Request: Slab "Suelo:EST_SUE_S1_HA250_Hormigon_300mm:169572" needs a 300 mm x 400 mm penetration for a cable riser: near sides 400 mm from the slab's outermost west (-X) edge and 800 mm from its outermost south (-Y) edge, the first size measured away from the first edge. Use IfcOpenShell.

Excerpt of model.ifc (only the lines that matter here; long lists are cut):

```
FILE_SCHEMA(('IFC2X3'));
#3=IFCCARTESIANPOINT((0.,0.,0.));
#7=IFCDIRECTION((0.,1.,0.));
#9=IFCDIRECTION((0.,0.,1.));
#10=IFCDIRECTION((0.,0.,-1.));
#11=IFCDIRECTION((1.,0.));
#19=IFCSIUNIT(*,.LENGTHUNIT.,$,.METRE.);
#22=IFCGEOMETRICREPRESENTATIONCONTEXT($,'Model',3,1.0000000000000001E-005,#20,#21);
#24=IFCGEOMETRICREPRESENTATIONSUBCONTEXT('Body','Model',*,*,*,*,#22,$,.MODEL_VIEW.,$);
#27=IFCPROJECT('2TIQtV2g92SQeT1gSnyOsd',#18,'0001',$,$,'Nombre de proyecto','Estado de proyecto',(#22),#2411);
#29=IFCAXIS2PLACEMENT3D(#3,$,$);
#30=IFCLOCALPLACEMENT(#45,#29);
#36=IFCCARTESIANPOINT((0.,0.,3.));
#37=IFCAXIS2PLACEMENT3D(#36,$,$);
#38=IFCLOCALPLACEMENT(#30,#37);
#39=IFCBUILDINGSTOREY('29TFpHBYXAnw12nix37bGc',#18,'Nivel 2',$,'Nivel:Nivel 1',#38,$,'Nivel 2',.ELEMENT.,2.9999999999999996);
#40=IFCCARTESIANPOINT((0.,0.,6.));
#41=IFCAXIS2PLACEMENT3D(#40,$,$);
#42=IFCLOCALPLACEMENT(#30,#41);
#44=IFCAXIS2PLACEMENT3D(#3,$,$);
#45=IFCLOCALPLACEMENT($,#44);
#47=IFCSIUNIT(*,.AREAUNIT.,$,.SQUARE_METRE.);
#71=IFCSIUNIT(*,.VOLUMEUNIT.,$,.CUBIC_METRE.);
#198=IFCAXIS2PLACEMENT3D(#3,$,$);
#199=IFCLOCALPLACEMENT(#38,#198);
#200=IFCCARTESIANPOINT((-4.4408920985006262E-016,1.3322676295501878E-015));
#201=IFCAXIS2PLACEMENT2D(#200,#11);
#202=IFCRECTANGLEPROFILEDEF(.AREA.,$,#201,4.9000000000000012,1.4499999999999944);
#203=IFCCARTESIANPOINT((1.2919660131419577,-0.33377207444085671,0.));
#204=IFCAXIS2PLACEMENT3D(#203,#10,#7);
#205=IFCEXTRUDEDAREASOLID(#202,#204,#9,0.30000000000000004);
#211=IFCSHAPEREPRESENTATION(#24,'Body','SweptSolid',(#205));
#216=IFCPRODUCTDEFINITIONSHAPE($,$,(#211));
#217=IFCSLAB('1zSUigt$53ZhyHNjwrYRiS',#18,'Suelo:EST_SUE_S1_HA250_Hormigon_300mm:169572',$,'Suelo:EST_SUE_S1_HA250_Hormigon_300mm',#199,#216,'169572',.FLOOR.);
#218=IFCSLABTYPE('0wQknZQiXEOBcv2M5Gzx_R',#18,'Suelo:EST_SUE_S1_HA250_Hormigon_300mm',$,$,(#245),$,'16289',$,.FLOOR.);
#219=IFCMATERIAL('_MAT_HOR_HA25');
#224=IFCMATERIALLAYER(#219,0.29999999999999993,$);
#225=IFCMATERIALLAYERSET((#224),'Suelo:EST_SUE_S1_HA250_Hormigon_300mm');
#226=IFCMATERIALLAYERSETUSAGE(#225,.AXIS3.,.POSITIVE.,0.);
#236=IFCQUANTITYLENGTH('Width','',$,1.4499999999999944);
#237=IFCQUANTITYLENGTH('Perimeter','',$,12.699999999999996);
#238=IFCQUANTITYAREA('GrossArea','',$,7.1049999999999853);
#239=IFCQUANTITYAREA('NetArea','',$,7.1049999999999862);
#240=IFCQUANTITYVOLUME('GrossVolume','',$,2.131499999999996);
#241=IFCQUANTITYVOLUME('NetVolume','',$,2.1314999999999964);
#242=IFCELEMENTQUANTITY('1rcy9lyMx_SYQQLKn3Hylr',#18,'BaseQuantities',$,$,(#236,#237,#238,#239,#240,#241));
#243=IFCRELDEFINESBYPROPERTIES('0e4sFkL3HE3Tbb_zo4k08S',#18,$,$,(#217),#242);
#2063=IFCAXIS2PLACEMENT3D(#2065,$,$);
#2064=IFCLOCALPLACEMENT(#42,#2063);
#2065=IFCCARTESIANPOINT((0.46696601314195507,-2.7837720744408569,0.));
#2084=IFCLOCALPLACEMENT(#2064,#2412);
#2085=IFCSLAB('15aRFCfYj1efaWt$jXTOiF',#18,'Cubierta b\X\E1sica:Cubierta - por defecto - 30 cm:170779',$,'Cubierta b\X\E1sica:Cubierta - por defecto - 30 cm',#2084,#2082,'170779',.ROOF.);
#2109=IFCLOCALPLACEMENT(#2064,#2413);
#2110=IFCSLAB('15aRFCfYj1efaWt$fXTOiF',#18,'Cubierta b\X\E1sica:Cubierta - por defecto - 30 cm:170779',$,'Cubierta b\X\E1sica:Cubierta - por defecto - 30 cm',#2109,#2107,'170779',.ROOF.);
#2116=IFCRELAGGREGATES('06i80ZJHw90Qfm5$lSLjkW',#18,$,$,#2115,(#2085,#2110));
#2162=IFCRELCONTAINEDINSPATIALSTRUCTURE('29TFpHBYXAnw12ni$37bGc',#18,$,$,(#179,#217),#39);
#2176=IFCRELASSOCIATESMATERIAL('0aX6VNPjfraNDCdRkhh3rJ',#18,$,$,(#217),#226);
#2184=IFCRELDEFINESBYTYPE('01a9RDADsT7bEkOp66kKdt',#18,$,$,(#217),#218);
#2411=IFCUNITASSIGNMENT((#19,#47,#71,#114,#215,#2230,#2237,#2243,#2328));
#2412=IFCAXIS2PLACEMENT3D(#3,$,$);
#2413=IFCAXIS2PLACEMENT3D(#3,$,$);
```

```python
import numpy as np
import ifcopenshell
import ifcopenshell.api.feature
import ifcopenshell.api.geometry
import ifcopenshell.api.pset
import ifcopenshell.api.root
import ifcopenshell.geom
import ifcopenshell.util.element
import ifcopenshell.util.placement
import ifcopenshell.util.representation
import ifcopenshell.util.shape
import ifcopenshell.util.unit

model = ifcopenshell.open("model.ifc")
unit_scale = ifcopenshell.util.unit.calculate_unit_scale(model)
area_scale = ifcopenshell.util.unit.calculate_unit_scale(model, "AREAUNIT")
volume_scale = ifcopenshell.util.unit.calculate_unit_scale(model, "VOLUMEUNIT")
settings = ifcopenshell.geom.settings()


def volume(element):
    """Net volume in cubic metres, openings subtracted."""
    shape = ifcopenshell.geom.create_shape(settings, element)
    return ifcopenshell.util.shape.get_volume(shape.geometry)


slab = model.by_guid("1zSUigt$53ZhyHNjwrYRiS")
before = volume(slab)

# Extent in the slab's own axes, in metres. The edges named are its -X and -Y sides.
slab_shape = ifcopenshell.geom.create_shape(settings, slab)
vertices = ifcopenshell.util.shape.get_vertices(slab_shape.geometry)
x_min, y_min, bottom = vertices.min(axis=0)
top = vertices[:, 2].max()

opening = ifcopenshell.api.root.create_entity(model, ifc_class="IfcOpeningElement", name="Cable riser opening")
context = ifcopenshell.util.representation.get_context(model, "Model", "Body", "MODEL_VIEW")
width, depth = 0.3, 0.4
outline = [(0.0, 0.0), (width, 0.0), (width, depth), (0.0, depth), (0.0, 0.0)]
# Overshoot both faces by 50 mm so the cut is clean.
shape = ifcopenshell.api.geometry.add_slab_representation(
    model, context=context, depth=top - bottom + 0.1, polyline=outline
)
ifcopenshell.api.geometry.assign_representation(model, product=opening, representation=shape)

matrix = ifcopenshell.util.placement.get_local_placement(slab.ObjectPlacement)
matrix[:, 3] = matrix @ np.append(np.array([x_min + 0.4, y_min + 0.8, bottom - 0.05]) / unit_scale, 1.0)
ifcopenshell.api.geometry.edit_object_placement(model, product=opening, matrix=matrix, is_si=False)
ifcopenshell.api.feature.add_feature(model, feature=opening, element=slab)

after = volume(slab)

# Update the slab's stored quantities.
qto = model.by_id(ifcopenshell.util.element.get_pset(slab, "BaseQuantities", should_inherit=False)["id"])
ifcopenshell.api.pset.edit_qto(model, qto=qto, properties={
    "NetArea": after / (top - bottom) / area_scale,
    "NetVolume": after / volume_scale,
})

print(f"slab volume {before:.3f} -> {after:.3f} m3")

model.write("model_updated.ifc")
```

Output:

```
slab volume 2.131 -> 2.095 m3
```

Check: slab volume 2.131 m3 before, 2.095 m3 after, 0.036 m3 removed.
